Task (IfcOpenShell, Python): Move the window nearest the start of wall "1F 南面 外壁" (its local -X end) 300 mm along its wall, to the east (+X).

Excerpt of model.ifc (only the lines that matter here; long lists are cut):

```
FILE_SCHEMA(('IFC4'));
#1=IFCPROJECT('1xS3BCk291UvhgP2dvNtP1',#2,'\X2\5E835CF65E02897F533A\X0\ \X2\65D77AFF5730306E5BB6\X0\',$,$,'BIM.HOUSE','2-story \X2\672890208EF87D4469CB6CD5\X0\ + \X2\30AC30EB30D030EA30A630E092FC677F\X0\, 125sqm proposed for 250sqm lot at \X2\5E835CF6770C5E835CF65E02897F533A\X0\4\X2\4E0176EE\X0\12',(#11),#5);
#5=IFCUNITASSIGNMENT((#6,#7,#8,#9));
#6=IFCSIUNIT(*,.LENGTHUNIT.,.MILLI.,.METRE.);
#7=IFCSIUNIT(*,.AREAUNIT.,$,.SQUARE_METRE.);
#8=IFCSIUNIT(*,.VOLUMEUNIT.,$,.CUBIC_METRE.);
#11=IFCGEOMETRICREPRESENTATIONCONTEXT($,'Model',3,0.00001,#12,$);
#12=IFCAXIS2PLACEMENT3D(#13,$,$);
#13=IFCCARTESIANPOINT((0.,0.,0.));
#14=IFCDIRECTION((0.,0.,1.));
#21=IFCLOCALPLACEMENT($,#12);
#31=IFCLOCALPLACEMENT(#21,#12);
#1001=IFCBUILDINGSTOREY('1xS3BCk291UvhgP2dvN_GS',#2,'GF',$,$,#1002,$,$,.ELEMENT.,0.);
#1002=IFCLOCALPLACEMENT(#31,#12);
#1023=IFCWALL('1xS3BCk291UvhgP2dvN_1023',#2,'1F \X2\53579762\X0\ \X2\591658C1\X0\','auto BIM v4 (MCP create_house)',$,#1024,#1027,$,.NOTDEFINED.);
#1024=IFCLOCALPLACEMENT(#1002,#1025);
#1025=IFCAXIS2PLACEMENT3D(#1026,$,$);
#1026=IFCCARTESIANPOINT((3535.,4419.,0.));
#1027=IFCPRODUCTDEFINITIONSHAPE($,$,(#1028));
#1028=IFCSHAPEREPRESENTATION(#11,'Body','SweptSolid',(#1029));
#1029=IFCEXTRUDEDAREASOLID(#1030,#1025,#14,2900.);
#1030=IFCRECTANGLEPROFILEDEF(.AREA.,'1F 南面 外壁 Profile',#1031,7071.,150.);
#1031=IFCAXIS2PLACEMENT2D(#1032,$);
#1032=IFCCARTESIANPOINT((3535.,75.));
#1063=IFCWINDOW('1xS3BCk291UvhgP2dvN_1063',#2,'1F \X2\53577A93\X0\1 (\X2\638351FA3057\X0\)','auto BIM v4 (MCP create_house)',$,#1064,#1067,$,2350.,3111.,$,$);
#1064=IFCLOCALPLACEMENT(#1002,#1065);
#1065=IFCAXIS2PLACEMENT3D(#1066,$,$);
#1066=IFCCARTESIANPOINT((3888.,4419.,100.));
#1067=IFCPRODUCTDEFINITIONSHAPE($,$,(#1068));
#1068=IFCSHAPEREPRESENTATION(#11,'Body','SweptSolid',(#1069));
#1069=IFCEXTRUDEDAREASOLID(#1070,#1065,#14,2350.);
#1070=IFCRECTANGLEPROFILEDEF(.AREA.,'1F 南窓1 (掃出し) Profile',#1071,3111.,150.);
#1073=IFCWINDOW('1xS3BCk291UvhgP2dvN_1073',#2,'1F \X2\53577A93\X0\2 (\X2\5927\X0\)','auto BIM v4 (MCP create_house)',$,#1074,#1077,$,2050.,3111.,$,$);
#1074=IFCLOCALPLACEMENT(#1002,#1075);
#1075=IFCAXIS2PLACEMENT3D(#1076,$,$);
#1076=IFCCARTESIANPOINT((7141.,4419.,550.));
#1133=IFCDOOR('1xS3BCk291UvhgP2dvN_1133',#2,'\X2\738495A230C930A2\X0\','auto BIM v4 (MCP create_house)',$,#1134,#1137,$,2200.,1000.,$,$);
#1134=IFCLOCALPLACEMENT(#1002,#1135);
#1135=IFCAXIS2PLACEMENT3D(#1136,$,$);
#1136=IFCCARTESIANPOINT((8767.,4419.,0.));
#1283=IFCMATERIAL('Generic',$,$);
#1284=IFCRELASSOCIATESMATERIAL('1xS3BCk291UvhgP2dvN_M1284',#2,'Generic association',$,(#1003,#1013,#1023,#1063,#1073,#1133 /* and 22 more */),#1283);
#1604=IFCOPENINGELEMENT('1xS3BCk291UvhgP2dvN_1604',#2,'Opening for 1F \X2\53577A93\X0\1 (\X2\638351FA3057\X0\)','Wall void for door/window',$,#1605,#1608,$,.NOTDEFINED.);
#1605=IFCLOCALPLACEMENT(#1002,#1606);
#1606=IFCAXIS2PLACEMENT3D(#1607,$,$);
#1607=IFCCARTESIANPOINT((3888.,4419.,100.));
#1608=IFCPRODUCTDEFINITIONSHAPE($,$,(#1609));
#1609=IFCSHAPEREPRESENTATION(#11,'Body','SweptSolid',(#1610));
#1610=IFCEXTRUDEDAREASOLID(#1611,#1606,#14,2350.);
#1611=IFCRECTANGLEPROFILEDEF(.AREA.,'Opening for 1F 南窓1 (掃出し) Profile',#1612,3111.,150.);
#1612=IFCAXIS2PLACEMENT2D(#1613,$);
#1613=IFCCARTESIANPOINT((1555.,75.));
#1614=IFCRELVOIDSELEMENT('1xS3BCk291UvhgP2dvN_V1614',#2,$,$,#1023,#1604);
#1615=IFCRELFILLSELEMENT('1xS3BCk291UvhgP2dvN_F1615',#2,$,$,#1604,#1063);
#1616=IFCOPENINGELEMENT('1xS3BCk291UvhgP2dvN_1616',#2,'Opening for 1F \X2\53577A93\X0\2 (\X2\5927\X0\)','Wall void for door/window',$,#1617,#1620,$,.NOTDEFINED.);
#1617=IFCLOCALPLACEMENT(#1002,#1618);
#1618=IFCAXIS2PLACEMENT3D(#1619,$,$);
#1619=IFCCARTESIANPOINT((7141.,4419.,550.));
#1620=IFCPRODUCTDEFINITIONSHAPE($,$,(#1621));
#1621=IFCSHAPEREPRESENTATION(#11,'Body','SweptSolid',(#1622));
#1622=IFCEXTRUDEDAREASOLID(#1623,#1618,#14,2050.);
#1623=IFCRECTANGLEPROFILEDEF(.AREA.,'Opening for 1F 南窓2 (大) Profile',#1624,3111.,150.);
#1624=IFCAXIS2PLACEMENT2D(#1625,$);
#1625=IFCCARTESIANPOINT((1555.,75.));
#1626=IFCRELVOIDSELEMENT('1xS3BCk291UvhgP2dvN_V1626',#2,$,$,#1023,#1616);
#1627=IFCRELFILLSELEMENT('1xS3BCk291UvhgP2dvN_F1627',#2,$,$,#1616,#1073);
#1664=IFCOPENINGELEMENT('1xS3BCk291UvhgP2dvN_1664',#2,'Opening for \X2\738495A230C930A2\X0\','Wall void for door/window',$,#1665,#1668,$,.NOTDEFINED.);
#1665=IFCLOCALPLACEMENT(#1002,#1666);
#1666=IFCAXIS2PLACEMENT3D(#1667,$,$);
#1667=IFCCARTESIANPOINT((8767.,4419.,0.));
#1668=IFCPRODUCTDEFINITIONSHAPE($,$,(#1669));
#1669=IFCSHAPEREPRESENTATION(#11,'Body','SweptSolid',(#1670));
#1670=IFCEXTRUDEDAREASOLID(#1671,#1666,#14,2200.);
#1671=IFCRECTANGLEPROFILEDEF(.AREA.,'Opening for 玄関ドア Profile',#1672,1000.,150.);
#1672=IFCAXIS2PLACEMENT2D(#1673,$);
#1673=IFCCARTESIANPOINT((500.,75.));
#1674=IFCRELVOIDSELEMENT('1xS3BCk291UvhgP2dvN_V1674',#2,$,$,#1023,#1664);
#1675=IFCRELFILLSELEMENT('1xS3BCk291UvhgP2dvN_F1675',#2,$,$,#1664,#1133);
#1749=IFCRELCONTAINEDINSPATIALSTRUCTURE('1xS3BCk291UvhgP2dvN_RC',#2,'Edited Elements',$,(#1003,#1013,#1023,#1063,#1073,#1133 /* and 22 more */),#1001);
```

```python
import ifcopenshell
import ifcopenshell.api.geometry
import ifcopenshell.util.placement
import ifcopenshell.util.unit

model = ifcopenshell.open("model.ifc")
unit_scale = ifcopenshell.util.unit.calculate_unit_scale(model)

window = model.by_guid("1xS3BCk291UvhgP2dvN_1063")
opening = window.FillsVoids[0].RelatingOpeningElement
wall = opening.VoidsElements[0].RelatingBuildingElement

wall_matrix = ifcopenshell.util.placement.get_local_placement(wall.ObjectPlacement)
shift = wall_matrix[:3, 0] * 0.3 / unit_scale
before = ifcopenshell.util.placement.get_local_placement(window.ObjectPlacement)[:3, 3].copy()

# The window is not placed relative to its opening, so move both.
for product in (opening, window):
    matrix = ifcopenshell.util.placement.get_local_placement(product.ObjectPlacement)
    matrix[:3, 3] += shift
    ifcopenshell.api.geometry.edit_object_placement(model, product=product, matrix=matrix, is_si=False)

after = ifcopenshell.util.placement.get_local_placement(window.ObjectPlacement)[:3, 3]
print("window moved by", (after - before).round(3) + 0.0)

model.write("model_rev.ifc")
```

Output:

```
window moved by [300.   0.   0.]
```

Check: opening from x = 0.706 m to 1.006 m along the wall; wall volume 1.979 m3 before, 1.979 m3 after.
